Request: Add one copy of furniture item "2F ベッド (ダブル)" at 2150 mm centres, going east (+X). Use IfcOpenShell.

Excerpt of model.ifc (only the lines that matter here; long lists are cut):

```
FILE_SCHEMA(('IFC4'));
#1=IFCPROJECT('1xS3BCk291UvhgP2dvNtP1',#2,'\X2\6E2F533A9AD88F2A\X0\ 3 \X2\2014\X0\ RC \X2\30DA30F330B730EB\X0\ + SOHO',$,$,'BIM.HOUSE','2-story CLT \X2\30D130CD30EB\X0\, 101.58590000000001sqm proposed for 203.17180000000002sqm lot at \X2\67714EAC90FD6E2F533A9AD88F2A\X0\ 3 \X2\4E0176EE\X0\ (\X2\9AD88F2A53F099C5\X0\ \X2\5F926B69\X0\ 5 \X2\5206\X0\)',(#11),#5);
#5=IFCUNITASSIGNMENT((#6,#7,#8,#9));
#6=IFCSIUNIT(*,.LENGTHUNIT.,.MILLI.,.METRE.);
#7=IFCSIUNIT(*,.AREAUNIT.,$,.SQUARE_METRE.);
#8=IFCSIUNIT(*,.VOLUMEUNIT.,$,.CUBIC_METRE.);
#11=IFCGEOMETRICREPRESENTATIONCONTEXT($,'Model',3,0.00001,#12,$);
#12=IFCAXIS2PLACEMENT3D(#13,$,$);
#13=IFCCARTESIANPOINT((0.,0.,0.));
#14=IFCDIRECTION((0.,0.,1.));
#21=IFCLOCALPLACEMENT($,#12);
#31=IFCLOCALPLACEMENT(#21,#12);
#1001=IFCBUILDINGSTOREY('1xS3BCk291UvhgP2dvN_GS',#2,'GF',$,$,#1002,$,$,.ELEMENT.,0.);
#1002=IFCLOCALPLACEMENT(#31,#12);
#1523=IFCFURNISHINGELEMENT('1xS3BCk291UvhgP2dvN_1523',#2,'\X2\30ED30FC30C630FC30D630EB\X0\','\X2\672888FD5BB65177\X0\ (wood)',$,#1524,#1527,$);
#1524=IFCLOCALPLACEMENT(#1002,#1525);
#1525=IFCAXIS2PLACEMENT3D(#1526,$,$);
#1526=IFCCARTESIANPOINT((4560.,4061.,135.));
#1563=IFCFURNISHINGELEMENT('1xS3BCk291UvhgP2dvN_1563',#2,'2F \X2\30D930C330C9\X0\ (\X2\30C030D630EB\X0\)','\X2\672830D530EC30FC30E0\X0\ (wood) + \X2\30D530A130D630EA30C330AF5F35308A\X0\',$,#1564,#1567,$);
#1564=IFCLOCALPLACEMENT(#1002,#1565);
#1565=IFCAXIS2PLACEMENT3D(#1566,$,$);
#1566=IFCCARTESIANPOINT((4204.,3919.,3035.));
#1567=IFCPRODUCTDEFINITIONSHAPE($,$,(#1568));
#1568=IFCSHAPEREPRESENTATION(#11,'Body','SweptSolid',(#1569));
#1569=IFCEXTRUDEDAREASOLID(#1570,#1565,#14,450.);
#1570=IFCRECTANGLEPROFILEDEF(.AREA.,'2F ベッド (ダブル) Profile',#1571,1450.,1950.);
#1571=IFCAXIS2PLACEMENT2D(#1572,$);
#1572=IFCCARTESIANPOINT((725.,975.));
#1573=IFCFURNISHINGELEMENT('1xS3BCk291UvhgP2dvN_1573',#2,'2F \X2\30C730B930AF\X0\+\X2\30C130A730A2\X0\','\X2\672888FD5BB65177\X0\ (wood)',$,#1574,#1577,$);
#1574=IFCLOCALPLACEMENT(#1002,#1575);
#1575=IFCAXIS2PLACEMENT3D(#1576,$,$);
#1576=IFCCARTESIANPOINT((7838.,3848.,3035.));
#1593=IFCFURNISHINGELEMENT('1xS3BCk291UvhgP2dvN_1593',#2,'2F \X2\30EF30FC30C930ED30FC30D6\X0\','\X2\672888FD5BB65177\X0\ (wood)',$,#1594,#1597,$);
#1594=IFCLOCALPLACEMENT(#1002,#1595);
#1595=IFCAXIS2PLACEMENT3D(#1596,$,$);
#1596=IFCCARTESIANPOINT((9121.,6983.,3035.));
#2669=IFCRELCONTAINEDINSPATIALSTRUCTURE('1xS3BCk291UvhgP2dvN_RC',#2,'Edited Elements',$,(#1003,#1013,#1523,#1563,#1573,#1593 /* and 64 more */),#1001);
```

```python
import numpy as np
import ifcopenshell
import ifcopenshell.api.geometry
import ifcopenshell.api.root
import ifcopenshell.util.element
import ifcopenshell.util.placement

model = ifcopenshell.open("model.ifc")


def reuse_history(source, copy):
    """copy_class also copies each property set's owner history, people and application; keep the originals."""
    for rel in copy.IsDefinedBy:
        if rel.is_a("IfcRelDefinesByProperties") and (history := rel.RelatingPropertyDefinition.OwnerHistory):
            rel.RelatingPropertyDefinition.OwnerHistory = source.OwnerHistory
            ifcopenshell.util.element.remove_deep2(model, history)


source = model.by_id(1563)
base = ifcopenshell.util.placement.get_local_placement(source.ObjectPlacement)
step = np.array([1.0, 0.0, 0.0]) * 2150.0

for i in range(1, 2):
    copy = ifcopenshell.api.root.copy_class(model, product=source)
    copy.Representation = ifcopenshell.util.element.copy_deep(
        model, source.Representation, exclude=["IfcGeometricRepresentationContext", "IfcRepresentationMap"]
    )
    reuse_history(source, copy)
    matrix = base.copy()
    matrix[:3, 3] += i * step
    print("added at", matrix[:3, 3].round(3) + 0.0)
    ifcopenshell.api.geometry.edit_object_placement(model, product=copy, matrix=matrix, is_si=False)

model.write("model_updated.ifc")
```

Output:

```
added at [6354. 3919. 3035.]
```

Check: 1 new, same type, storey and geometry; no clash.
